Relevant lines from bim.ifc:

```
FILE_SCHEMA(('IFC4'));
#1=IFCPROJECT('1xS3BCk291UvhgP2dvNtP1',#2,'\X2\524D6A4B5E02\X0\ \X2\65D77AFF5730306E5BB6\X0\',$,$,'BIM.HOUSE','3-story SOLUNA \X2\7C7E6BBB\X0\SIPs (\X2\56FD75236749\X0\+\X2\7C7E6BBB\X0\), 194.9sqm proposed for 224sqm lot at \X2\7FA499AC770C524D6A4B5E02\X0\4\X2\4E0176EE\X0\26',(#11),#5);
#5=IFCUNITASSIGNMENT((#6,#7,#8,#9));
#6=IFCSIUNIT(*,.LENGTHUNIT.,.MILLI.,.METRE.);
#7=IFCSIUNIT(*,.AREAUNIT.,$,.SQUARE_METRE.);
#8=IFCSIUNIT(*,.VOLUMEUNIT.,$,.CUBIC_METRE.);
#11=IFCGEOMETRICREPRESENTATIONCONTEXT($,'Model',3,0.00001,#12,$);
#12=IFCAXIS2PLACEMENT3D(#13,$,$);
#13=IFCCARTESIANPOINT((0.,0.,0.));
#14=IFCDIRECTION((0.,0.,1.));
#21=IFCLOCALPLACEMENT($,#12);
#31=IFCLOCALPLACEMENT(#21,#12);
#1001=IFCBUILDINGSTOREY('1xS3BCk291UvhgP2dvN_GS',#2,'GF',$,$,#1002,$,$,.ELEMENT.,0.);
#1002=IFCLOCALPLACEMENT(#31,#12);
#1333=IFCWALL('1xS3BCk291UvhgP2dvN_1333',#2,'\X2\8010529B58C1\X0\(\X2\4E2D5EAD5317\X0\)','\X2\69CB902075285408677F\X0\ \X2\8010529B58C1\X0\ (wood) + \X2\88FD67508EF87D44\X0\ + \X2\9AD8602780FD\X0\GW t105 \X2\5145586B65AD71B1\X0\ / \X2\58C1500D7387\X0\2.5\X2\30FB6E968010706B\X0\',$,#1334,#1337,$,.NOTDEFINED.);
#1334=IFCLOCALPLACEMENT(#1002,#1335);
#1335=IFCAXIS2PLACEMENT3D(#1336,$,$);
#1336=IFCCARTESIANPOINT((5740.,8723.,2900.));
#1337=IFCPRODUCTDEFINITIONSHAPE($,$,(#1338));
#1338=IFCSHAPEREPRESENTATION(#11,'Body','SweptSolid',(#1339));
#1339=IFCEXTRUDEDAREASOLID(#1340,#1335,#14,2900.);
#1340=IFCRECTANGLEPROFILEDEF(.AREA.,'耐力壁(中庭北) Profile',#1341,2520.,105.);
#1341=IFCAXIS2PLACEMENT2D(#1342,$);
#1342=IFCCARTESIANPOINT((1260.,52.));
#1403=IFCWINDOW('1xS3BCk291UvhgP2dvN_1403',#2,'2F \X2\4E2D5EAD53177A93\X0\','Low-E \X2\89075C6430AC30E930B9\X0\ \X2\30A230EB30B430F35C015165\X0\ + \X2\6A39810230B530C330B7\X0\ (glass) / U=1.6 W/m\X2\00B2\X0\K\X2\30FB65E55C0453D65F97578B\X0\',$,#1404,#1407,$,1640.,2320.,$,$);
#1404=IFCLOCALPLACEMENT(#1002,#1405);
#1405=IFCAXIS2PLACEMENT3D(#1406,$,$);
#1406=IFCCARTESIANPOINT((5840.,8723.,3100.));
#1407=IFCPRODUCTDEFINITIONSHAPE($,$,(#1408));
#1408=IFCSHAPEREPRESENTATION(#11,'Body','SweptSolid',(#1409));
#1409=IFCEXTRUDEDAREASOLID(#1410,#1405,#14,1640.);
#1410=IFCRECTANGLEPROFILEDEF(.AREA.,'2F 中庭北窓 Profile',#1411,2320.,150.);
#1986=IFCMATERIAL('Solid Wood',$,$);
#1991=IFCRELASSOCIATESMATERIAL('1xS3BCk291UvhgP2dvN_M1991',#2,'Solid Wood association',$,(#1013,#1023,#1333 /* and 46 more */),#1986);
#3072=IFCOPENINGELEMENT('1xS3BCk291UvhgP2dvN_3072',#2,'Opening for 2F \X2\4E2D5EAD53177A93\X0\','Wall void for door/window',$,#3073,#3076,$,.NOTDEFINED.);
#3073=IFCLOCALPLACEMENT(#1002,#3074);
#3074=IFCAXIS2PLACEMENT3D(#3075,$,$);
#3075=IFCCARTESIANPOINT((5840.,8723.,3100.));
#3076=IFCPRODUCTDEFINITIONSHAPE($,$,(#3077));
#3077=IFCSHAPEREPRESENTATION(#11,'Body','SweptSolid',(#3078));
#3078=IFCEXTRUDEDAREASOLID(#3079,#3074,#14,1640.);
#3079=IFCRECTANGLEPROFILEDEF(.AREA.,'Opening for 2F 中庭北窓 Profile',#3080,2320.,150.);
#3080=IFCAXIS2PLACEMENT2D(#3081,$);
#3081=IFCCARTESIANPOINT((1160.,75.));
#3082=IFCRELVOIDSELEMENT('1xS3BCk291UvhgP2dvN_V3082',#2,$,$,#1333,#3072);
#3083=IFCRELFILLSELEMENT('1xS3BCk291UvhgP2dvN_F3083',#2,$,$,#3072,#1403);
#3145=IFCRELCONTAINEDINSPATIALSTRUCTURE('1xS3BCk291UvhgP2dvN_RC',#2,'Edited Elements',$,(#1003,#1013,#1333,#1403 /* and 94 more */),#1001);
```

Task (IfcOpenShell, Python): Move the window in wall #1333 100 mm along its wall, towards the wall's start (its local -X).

```python
import ifcopenshell
import ifcopenshell.api.geometry
import ifcopenshell.util.placement

model = ifcopenshell.open("bim.ifc")

window = model.by_guid("1xS3BCk291UvhgP2dvN_1403")
opening = window.FillsVoids[0].RelatingOpeningElement
wall = opening.VoidsElements[0].RelatingBuildingElement

wall_matrix = ifcopenshell.util.placement.get_local_placement(wall.ObjectPlacement)
shift = wall_matrix[:3, 0] * -100.0
before = ifcopenshell.util.placement.get_local_placement(window.ObjectPlacement)[:3, 3].copy()

# The window is not placed relative to its opening, so move both.
for product in (opening, window):
    matrix = ifcopenshell.util.placement.get_local_placement(product.ObjectPlacement)
    matrix[:3, 3] += shift
    ifcopenshell.api.geometry.edit_object_placement(model, product=product, matrix=matrix, is_si=False)

after = ifcopenshell.util.placement.get_local_placement(window.ObjectPlacement)[:3, 3]
print("window moved by", (after - before).round(3) + 0.0)

model.write("bim_rev.ifc")
```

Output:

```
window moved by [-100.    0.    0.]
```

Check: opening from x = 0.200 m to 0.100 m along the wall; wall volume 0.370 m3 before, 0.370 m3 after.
